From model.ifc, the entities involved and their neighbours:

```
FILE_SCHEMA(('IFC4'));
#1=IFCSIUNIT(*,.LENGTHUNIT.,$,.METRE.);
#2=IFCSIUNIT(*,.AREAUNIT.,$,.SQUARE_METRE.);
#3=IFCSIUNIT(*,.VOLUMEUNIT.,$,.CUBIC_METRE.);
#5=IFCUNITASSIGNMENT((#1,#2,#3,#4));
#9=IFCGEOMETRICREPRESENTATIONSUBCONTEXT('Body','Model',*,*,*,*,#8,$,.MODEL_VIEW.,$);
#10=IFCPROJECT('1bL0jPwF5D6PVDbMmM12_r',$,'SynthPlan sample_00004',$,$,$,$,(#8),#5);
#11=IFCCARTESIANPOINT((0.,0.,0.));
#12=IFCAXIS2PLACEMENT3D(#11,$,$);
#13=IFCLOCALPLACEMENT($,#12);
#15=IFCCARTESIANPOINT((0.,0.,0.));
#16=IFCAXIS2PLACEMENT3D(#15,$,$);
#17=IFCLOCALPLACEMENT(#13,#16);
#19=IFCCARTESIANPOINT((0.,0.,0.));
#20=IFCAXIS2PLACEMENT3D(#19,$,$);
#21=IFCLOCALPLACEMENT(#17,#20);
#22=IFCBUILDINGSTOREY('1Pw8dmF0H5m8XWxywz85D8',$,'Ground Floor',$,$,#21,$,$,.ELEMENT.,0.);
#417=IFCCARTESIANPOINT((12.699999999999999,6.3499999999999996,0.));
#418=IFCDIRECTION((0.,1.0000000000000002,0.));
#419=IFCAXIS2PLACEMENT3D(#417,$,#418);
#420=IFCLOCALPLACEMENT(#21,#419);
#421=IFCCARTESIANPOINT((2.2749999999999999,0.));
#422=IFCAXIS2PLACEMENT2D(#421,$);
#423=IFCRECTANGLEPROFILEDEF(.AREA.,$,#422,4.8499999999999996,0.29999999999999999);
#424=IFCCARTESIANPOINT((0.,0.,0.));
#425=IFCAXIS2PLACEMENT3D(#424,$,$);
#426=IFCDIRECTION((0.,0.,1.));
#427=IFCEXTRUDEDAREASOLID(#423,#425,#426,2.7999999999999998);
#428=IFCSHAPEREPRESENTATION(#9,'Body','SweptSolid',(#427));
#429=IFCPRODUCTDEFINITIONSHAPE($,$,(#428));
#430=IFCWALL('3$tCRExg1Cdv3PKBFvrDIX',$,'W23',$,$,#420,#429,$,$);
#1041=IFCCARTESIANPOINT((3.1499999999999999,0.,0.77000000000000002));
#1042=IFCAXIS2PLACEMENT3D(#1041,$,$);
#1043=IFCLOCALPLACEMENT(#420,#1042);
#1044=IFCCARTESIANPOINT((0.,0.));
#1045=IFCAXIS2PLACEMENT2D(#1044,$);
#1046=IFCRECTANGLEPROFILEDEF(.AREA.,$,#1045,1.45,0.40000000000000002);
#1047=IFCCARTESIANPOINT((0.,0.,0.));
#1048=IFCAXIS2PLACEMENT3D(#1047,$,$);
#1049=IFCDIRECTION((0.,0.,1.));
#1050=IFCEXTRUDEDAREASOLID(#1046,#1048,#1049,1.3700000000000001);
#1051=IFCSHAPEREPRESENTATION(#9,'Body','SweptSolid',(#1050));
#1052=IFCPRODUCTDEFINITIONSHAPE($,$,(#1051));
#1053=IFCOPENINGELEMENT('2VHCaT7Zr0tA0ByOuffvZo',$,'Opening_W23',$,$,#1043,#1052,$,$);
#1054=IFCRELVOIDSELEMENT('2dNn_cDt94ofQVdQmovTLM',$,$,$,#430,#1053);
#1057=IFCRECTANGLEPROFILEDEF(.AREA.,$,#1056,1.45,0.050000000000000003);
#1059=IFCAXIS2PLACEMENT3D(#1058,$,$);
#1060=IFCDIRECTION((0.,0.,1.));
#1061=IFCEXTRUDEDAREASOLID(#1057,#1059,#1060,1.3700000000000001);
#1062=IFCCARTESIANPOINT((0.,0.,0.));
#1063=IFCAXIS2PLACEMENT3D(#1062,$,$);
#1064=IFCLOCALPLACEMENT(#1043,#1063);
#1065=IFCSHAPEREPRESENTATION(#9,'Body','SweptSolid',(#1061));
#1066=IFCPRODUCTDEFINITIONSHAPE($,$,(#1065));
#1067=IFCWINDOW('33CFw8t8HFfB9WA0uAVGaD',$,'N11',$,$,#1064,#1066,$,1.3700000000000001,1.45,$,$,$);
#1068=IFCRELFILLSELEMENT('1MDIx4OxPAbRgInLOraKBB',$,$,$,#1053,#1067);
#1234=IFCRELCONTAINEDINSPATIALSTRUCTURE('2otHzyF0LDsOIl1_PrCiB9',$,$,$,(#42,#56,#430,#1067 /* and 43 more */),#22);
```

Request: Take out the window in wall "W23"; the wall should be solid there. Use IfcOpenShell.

```python
import ifcopenshell
import ifcopenshell.api.feature
import ifcopenshell.api.root
import ifcopenshell.geom
import ifcopenshell.util.shape

model = ifcopenshell.open("model.ifc")
settings = ifcopenshell.geom.settings()


def volume(element):
    """Net volume in cubic metres, openings subtracted."""
    shape = ifcopenshell.geom.create_shape(settings, element)
    return ifcopenshell.util.shape.get_volume(shape.geometry)


window = model.by_guid("33CFw8t8HFfB9WA0uAVGaD")
opening = window.FillsVoids[0].RelatingOpeningElement
wall = opening.VoidsElements[0].RelatingBuildingElement
before = volume(wall)

ifcopenshell.api.root.remove_product(model, product=window)
ifcopenshell.api.feature.remove_feature(model, feature=opening)

after = volume(wall)

print(f"wall volume {before:.3f} -> {after:.3f} m3")

model.write("model_rev.ifc")
```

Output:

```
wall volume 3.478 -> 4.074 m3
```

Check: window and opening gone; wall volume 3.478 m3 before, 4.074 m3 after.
